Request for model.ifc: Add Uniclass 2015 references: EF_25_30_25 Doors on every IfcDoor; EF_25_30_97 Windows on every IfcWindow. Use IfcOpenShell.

First a look at what the model holds.

```python
import ifcopenshell

model = ifcopenshell.open("model.ifc")
print(model.schema)
print("classifications:", [c.Name for c in model.by_type("IfcClassification")])
for ifc_class in ("IfcDoor", "IfcRoof", "IfcStair", "IfcWall", "IfcWindow"):
    print(ifc_class, len(model.by_type(ifc_class)))
```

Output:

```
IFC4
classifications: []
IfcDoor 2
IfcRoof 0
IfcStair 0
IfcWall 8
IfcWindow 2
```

```python
import ifcopenshell
import ifcopenshell.api.classification

model = ifcopenshell.open("model.ifc")

system = ifcopenshell.api.classification.add_classification(model, classification="Uniclass 2015")

codes = {
    "IfcDoor": ("EF_25_30_25", "Doors"),
    "IfcWindow": ("EF_25_30_97", "Windows"),
}
for ifc_class, (code, name) in codes.items():
    products = model.by_type(ifc_class)
    ifcopenshell.api.classification.add_reference(
        model, products=products, classification=system, identification=code, name=name
    )
    print(code, len(products))

model.write("model_rev.ifc")
```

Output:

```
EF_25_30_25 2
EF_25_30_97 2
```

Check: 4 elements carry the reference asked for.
